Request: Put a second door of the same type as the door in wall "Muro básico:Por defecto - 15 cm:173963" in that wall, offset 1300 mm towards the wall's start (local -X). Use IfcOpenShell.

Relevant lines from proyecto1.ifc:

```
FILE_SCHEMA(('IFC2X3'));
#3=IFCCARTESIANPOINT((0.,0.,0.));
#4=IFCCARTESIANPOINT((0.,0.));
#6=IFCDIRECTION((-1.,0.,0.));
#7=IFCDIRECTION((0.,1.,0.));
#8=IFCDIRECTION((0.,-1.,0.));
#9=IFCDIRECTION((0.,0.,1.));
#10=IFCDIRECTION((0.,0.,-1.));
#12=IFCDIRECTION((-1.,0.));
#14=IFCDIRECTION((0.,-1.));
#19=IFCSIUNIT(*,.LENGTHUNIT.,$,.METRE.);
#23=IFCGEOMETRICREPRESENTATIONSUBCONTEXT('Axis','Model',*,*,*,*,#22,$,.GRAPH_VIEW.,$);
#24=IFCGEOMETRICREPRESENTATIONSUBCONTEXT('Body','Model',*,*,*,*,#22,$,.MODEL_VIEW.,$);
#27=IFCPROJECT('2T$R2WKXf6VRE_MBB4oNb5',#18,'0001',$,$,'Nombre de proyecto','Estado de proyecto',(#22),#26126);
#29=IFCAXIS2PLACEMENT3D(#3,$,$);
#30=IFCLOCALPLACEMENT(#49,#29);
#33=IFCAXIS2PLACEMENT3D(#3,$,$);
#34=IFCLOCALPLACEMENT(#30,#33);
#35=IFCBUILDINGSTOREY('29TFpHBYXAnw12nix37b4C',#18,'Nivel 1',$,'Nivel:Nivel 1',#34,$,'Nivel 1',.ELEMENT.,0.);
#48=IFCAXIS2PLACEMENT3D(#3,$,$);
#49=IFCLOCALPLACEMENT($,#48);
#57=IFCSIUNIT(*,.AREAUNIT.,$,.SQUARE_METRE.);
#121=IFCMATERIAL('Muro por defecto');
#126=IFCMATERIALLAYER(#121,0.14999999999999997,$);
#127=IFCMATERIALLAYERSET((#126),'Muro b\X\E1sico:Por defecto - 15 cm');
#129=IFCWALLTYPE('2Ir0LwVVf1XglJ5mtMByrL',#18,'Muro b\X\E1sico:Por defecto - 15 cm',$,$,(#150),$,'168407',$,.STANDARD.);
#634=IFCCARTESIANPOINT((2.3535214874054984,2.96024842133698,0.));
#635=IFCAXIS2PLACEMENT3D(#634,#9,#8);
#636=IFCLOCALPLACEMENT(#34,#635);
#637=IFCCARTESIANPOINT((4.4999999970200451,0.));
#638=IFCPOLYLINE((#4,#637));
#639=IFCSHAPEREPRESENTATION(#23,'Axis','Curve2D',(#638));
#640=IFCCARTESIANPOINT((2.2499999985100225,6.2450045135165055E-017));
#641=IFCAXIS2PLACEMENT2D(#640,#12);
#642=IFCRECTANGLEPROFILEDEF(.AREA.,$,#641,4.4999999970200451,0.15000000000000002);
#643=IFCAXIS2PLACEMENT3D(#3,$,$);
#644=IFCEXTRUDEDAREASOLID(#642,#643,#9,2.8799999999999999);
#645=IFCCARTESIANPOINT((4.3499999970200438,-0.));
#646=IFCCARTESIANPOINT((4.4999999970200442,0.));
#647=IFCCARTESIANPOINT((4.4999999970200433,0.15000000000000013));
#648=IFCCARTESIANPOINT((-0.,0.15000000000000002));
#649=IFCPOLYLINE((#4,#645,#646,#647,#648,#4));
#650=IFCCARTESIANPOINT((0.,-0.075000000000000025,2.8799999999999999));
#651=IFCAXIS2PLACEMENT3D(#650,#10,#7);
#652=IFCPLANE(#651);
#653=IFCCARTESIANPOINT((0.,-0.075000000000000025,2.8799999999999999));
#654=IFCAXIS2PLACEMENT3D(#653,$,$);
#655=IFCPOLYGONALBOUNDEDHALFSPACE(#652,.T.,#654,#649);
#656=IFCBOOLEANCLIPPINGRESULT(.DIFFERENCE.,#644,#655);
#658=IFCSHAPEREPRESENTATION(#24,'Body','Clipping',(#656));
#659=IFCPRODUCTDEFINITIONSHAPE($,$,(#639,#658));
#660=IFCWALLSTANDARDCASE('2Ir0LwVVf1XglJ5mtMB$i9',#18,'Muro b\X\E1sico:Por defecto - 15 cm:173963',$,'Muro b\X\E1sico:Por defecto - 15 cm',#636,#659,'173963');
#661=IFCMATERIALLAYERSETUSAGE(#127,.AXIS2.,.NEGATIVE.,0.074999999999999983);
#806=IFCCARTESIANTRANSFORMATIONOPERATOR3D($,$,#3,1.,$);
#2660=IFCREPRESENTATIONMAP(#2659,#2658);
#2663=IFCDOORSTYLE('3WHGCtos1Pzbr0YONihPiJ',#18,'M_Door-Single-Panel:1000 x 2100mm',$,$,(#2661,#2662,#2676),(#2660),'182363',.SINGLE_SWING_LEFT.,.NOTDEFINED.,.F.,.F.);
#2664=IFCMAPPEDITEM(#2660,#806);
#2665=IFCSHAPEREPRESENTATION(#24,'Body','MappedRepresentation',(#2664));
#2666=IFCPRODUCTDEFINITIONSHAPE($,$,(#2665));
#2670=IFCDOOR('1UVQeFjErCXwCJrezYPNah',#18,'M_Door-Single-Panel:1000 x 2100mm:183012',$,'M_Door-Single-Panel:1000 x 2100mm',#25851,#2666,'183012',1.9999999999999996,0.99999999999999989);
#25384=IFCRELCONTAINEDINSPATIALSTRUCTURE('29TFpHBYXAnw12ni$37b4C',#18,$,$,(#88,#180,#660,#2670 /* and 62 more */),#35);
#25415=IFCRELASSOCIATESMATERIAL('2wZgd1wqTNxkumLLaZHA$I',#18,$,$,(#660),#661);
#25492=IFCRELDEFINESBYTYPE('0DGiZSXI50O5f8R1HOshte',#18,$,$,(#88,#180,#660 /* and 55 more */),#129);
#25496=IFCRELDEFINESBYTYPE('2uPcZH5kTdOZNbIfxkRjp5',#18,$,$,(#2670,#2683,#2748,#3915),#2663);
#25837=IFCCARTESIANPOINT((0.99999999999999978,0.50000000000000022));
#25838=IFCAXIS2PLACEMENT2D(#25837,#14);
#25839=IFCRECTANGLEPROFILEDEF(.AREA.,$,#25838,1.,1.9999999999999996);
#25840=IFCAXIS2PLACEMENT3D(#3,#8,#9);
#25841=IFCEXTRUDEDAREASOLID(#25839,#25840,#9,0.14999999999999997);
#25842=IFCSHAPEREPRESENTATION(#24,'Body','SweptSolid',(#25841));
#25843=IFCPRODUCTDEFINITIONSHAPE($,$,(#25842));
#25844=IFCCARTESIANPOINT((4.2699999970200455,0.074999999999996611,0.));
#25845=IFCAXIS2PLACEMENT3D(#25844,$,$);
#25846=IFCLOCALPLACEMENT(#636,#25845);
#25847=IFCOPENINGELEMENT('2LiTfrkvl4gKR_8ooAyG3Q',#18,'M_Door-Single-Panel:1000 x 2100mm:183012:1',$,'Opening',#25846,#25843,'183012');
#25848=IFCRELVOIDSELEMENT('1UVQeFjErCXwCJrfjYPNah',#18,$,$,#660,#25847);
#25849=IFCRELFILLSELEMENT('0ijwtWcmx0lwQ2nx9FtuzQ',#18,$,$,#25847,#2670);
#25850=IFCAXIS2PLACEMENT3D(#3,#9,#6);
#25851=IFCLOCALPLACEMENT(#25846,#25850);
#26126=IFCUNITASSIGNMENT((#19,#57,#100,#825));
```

```python
import ifcopenshell
import ifcopenshell.api.feature
import ifcopenshell.api.geometry
import ifcopenshell.api.root
import ifcopenshell.geom
import ifcopenshell.util.element
import ifcopenshell.util.placement
import ifcopenshell.util.shape

model = ifcopenshell.open("proyecto1.ifc")
settings = ifcopenshell.geom.settings()


def volume(element):
    """Net volume in cubic metres, openings subtracted."""
    shape = ifcopenshell.geom.create_shape(settings, element)
    return ifcopenshell.util.shape.get_volume(shape.geometry)


def reuse_history(source, copy):
    """copy_class also copies each property set's owner history, people and application; keep the originals."""
    for rel in copy.IsDefinedBy:
        if rel.is_a("IfcRelDefinesByProperties") and (history := rel.RelatingPropertyDefinition.OwnerHistory):
            rel.RelatingPropertyDefinition.OwnerHistory = source.OwnerHistory
            ifcopenshell.util.element.remove_deep2(model, history)


door = model.by_guid("1UVQeFjErCXwCJrezYPNah")
opening = door.FillsVoids[0].RelatingOpeningElement
wall = opening.VoidsElements[0].RelatingBuildingElement
before = volume(wall)
shift = ifcopenshell.util.placement.get_local_placement(wall.ObjectPlacement)[:3, 0] * -1.3

# copy_class copies the void relationship, type, container and properties, but no geometry.
new_opening = ifcopenshell.api.root.copy_class(model, product=opening)
new_opening.Representation = ifcopenshell.util.element.copy_deep(
    model, opening.Representation, exclude=["IfcGeometricRepresentationContext", "IfcRepresentationMap"]
)
new_opening.Name = "M_Door-Single-Panel:1000 x 2100mm"
new_opening.Tag = None
new_door = ifcopenshell.api.root.copy_class(model, product=door)
new_door.Representation = ifcopenshell.util.element.copy_deep(
    model, door.Representation, exclude=["IfcGeometricRepresentationContext", "IfcRepresentationMap"]
)
new_door.Name = "M_Door-Single-Panel:1000 x 2100mm"
new_door.Tag = None
reuse_history(door, new_door)
fills = ifcopenshell.api.feature.add_filling(model, opening=new_opening, element=new_door)
fills.OwnerHistory = new_door.OwnerHistory  # required in IFC2X3

for old, new in ((opening, new_opening), (door, new_door)):
    matrix = ifcopenshell.util.placement.get_local_placement(old.ObjectPlacement)
    matrix[:3, 3] += shift
    ifcopenshell.api.geometry.edit_object_placement(model, product=new, matrix=matrix, is_si=False)

after = volume(wall)

print(f"wall volume {before:.3f} -> {after:.3f} m3")

model.write("proyecto1-out.ifc")
```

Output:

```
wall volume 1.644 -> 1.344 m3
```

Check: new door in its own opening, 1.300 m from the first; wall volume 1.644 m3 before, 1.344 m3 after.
